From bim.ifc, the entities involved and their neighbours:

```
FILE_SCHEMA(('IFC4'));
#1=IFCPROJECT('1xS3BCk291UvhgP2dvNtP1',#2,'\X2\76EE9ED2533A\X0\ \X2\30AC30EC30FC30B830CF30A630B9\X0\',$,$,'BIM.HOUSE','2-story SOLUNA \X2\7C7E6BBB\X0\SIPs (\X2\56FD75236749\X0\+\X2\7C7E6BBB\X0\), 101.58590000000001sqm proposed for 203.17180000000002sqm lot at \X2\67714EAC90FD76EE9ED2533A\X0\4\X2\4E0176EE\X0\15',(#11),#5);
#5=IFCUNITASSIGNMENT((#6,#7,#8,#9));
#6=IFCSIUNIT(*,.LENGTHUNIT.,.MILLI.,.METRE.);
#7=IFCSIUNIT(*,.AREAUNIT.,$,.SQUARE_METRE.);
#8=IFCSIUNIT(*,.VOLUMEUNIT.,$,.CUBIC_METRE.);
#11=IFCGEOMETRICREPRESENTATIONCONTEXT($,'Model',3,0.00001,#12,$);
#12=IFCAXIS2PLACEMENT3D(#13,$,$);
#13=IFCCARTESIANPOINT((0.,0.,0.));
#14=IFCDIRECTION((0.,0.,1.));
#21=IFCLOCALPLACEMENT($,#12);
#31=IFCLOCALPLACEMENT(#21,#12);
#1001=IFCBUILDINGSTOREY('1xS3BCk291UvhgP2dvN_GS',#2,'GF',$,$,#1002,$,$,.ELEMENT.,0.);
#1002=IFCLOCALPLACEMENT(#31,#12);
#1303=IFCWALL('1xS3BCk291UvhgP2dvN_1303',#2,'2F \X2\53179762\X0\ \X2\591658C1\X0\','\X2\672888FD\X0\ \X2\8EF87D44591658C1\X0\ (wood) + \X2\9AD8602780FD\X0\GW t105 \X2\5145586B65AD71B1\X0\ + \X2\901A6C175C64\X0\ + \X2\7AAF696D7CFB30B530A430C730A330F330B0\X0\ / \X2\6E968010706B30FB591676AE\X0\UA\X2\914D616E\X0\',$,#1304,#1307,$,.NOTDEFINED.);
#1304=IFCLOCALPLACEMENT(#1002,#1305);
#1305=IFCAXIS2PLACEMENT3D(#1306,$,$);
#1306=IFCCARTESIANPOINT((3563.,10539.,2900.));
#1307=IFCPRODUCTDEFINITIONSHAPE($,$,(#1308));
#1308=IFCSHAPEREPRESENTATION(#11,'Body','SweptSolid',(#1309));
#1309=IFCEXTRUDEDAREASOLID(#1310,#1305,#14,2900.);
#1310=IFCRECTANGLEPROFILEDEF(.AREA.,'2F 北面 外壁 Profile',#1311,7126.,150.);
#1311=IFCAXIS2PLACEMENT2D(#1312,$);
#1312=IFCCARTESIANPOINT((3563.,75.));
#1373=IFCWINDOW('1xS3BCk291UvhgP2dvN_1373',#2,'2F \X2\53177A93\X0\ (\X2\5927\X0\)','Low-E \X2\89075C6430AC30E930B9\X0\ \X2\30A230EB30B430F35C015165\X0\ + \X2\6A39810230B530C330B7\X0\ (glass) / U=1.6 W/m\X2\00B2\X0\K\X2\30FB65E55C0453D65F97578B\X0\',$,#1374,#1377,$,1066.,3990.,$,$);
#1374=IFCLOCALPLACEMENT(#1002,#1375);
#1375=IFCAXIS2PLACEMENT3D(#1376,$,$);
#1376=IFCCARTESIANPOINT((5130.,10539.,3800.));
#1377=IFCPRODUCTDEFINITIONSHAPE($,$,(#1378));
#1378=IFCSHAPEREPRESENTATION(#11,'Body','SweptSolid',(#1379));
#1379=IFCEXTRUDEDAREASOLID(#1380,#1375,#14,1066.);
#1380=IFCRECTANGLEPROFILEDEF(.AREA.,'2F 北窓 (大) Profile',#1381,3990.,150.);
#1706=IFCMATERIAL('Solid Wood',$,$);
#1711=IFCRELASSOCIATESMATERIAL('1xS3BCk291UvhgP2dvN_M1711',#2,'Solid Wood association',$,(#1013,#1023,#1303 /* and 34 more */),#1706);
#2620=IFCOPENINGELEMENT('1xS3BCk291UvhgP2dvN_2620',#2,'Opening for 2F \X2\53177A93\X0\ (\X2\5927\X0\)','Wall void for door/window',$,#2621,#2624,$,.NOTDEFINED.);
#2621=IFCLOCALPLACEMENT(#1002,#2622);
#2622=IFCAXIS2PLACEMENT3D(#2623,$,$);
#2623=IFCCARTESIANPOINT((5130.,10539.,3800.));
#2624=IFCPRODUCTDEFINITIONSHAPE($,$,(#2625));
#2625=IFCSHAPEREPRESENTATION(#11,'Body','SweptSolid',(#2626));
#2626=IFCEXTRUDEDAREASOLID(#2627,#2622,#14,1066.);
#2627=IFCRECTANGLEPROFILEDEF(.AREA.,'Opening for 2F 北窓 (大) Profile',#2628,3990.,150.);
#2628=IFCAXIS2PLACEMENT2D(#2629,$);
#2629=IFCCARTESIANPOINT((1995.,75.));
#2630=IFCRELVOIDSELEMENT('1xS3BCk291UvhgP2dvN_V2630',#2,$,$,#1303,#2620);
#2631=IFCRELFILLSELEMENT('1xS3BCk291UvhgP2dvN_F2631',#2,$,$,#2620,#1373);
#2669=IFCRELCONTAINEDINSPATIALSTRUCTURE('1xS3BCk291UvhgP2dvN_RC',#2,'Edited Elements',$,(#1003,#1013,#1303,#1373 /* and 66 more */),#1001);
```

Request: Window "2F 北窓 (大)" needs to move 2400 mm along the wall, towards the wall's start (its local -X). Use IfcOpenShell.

```python
import ifcopenshell
import ifcopenshell.api.geometry
import ifcopenshell.util.placement

model = ifcopenshell.open("bim.ifc")

window = model.by_id(1373)
opening = window.FillsVoids[0].RelatingOpeningElement
wall = opening.VoidsElements[0].RelatingBuildingElement

wall_matrix = ifcopenshell.util.placement.get_local_placement(wall.ObjectPlacement)
shift = wall_matrix[:3, 0] * -2400.0
before = ifcopenshell.util.placement.get_local_placement(window.ObjectPlacement)[:3, 3].copy()

# The window is not placed relative to its opening, so move both.
for product in (opening, window):
    matrix = ifcopenshell.util.placement.get_local_placement(product.ObjectPlacement)
    matrix[:3, 3] += shift
    ifcopenshell.api.geometry.edit_object_placement(model, product=product, matrix=matrix, is_si=False)

after = ifcopenshell.util.placement.get_local_placement(window.ObjectPlacement)[:3, 3]
print("window moved by", (after - before).round(3) + 0.0)

model.write("bim_v2.ifc")
```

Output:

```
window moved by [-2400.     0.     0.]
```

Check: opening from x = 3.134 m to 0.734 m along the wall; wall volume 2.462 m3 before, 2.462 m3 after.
